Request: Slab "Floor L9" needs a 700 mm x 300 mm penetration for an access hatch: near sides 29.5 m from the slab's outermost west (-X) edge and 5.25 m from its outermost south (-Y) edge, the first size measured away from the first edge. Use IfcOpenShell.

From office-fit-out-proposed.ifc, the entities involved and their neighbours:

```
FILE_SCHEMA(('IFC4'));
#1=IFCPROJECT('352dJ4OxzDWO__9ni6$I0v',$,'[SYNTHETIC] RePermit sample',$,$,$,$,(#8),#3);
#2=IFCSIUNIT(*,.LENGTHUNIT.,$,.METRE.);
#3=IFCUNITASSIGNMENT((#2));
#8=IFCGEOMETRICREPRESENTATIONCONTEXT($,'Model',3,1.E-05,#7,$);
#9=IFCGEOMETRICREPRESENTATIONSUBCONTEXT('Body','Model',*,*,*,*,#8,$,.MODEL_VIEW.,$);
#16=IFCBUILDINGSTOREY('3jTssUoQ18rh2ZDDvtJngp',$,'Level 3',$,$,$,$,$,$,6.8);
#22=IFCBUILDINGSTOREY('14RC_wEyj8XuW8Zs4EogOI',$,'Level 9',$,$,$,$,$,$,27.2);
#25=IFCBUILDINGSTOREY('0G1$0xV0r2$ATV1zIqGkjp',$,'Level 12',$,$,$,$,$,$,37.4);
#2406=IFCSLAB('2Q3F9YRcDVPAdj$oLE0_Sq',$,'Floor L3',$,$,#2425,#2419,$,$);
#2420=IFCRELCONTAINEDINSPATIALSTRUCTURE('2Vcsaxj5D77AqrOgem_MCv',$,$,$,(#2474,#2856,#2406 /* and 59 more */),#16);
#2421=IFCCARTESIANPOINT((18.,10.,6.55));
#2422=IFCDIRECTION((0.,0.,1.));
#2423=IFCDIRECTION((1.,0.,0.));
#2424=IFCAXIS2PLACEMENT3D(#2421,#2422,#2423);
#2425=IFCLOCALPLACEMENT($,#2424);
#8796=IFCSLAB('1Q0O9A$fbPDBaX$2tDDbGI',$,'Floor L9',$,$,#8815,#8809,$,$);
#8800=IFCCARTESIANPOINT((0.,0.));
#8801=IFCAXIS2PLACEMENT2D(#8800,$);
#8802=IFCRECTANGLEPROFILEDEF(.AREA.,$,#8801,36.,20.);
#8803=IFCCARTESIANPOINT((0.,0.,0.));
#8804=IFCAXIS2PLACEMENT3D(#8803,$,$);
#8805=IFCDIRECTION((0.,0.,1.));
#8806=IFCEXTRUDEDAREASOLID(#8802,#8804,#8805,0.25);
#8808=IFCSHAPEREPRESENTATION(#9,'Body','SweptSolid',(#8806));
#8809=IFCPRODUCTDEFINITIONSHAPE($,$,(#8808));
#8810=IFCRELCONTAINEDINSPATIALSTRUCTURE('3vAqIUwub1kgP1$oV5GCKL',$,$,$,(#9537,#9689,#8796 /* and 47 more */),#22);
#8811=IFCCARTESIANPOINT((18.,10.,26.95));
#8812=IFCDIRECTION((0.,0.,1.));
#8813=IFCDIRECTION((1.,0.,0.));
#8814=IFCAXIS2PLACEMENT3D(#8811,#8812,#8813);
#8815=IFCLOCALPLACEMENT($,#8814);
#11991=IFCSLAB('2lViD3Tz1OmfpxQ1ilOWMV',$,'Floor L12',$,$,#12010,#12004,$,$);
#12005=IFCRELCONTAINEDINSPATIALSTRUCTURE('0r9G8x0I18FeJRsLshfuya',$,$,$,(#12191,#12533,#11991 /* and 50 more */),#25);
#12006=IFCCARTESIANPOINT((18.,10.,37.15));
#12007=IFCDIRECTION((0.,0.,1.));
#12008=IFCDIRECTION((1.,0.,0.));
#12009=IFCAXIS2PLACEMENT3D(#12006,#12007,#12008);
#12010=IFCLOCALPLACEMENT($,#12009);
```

```python
import numpy as np
import ifcopenshell
import ifcopenshell.api.feature
import ifcopenshell.api.geometry
import ifcopenshell.api.root
import ifcopenshell.geom
import ifcopenshell.util.placement
import ifcopenshell.util.representation
import ifcopenshell.util.shape
import ifcopenshell.util.unit

model = ifcopenshell.open("office-fit-out-proposed.ifc")
unit_scale = ifcopenshell.util.unit.calculate_unit_scale(model)
settings = ifcopenshell.geom.settings()


def volume(element):
    """Net volume in cubic metres, openings subtracted."""
    shape = ifcopenshell.geom.create_shape(settings, element)
    return ifcopenshell.util.shape.get_volume(shape.geometry)


slab = model.by_guid("1Q0O9A$fbPDBaX$2tDDbGI")
before = volume(slab)

# Extent in the slab's own axes, in metres. The edges named are its -X and -Y sides.
slab_shape = ifcopenshell.geom.create_shape(settings, slab)
vertices = ifcopenshell.util.shape.get_vertices(slab_shape.geometry)
x_min, y_min, bottom = vertices.min(axis=0)
top = vertices[:, 2].max()

opening = ifcopenshell.api.root.create_entity(model, ifc_class="IfcOpeningElement", name="Access hatch opening", predefined_type="OPENING")
context = ifcopenshell.util.representation.get_context(model, "Model", "Body", "MODEL_VIEW")
width, depth = 0.7, 0.3
outline = [(0.0, 0.0), (width, 0.0), (width, depth), (0.0, depth), (0.0, 0.0)]
# Overshoot both faces by 50 mm so the cut is clean.
shape = ifcopenshell.api.geometry.add_slab_representation(
    model, context=context, depth=top - bottom + 0.1, polyline=outline
)
ifcopenshell.api.geometry.assign_representation(model, product=opening, representation=shape)

matrix = ifcopenshell.util.placement.get_local_placement(slab.ObjectPlacement)
matrix[:, 3] = matrix @ np.append(np.array([x_min + 29.5, y_min + 5.25, bottom - 0.05]) / unit_scale, 1.0)
ifcopenshell.api.geometry.edit_object_placement(model, product=opening, matrix=matrix, is_si=False)
ifcopenshell.api.feature.add_feature(model, feature=opening, element=slab)

after = volume(slab)

print(f"slab volume {before:.3f} -> {after:.3f} m3")

model.write("office-fit-out-proposed-out.ifc")
```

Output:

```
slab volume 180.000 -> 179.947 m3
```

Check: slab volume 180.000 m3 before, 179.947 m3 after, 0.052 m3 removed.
